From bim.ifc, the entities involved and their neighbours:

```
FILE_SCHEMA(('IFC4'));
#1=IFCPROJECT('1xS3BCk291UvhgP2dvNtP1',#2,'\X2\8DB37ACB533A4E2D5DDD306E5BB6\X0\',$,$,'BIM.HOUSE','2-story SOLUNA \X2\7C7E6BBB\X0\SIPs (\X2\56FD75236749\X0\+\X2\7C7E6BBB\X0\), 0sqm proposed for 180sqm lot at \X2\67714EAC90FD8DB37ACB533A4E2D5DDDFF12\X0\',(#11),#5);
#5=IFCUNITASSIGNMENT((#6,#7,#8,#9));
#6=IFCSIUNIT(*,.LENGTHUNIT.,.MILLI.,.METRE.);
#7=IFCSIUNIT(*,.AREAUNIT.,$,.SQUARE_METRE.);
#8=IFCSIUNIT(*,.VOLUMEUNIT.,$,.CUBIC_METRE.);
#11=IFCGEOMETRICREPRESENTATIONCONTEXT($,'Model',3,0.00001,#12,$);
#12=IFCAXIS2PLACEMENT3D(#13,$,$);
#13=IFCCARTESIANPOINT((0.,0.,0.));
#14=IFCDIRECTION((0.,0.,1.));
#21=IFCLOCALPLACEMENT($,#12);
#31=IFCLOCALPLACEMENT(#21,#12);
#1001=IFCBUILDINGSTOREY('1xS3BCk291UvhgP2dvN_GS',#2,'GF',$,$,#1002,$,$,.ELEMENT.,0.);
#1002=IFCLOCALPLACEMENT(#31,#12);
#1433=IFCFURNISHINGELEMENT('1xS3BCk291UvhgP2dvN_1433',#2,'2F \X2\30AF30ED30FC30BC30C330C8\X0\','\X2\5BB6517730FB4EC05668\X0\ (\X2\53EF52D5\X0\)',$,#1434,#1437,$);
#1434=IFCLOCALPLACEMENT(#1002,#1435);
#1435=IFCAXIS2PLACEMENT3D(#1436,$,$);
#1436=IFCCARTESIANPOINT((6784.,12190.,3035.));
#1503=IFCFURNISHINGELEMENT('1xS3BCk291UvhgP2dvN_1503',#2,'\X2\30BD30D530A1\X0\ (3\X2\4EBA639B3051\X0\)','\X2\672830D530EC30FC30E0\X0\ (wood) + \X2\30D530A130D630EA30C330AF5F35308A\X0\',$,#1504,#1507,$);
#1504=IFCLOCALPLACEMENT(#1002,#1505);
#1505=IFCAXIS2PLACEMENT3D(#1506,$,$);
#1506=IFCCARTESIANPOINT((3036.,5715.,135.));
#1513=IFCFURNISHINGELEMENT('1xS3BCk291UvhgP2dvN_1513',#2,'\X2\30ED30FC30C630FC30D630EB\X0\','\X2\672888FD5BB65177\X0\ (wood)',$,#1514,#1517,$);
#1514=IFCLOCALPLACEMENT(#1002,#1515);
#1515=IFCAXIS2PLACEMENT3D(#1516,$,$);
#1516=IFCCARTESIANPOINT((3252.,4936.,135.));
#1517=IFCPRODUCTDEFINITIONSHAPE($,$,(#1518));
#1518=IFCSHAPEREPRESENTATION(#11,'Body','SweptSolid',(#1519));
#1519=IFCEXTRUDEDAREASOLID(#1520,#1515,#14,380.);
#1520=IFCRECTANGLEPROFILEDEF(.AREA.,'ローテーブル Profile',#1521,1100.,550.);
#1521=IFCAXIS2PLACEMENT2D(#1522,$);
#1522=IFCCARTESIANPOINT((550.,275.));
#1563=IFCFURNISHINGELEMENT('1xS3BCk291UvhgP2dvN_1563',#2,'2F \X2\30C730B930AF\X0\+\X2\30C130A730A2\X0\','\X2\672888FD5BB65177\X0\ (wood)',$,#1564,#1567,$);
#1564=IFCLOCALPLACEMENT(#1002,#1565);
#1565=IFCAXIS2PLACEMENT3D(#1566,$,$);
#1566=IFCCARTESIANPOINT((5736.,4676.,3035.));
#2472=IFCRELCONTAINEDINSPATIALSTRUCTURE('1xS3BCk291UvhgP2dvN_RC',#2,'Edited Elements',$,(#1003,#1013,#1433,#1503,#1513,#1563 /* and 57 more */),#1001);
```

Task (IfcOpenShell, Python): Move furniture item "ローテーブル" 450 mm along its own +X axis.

```python
import ifcopenshell
import ifcopenshell.api.geometry
import ifcopenshell.util.placement
import ifcopenshell.util.unit

model = ifcopenshell.open("bim.ifc")
unit_scale = ifcopenshell.util.unit.calculate_unit_scale(model)

item = model.by_id(1513)
matrix = ifcopenshell.util.placement.get_local_placement(item.ObjectPlacement)
matrix[:3, 3] += matrix[:3, 0] * 0.45 / unit_scale
ifcopenshell.api.geometry.edit_object_placement(model, product=item, matrix=matrix, is_si=False)

print(ifcopenshell.util.placement.get_local_placement(item.ObjectPlacement).round(3) + 0.0)

model.write("bim_rev.ifc")
```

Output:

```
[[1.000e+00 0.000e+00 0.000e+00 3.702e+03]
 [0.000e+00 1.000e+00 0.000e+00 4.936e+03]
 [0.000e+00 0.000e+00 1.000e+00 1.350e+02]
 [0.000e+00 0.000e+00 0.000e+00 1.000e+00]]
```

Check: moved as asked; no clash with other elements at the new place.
